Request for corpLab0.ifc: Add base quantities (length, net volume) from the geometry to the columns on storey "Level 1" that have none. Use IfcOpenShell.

First a look at what the model holds.

```python
import ifcopenshell
import ifcopenshell.util.element
import ifcopenshell.util.unit

model = ifcopenshell.open("corpLab0.ifc")
print(model.schema)
for unit_type in ("LENGTHUNIT", "AREAUNIT", "VOLUMEUNIT"):
    print(unit_type, ifcopenshell.util.unit.calculate_unit_scale(model, unit_type))
storey = next(s for s in model.by_type("IfcBuildingStorey") if s.Name == "Level 1")
columns = [e for e in ifcopenshell.util.element.get_decomposition(storey) if e.is_a("IfcColumn")]
for e in sorted(columns, key=lambda e: e.id()):
    print(e.id(), e.is_a(), e.Name, list(ifcopenshell.util.element.get_psets(e, qtos_only=True)), sep=" | ")
```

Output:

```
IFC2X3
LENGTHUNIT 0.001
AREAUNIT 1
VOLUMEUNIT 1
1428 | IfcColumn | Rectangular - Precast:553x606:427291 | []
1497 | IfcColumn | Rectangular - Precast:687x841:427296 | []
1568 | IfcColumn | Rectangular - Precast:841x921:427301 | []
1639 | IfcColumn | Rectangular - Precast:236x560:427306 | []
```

```python
import ifcopenshell
import ifcopenshell.api.pset
import ifcopenshell.geom
import ifcopenshell.util.element
import ifcopenshell.util.shape
import ifcopenshell.util.unit

model = ifcopenshell.open("corpLab0.ifc")
unit_scale = ifcopenshell.util.unit.calculate_unit_scale(model)
volume_scale = ifcopenshell.util.unit.calculate_unit_scale(model, "VOLUMEUNIT")
settings = ifcopenshell.geom.settings()

storey = next(s for s in model.by_type("IfcBuildingStorey") if s.Name == "Level 1")
columns = [e for e in ifcopenshell.util.element.get_decomposition(storey) if e.is_a("IfcColumn")]

for e in sorted(columns, key=lambda e: e.id()):
    if ifcopenshell.util.element.get_psets(e, qtos_only=True, should_inherit=False):
        continue
    # Geometry comes back in metres, in the element's own axes.
    shape = ifcopenshell.geom.create_shape(settings, e)
    values = {
        "Length": ifcopenshell.util.shape.get_z(shape.geometry) / unit_scale,
        "NetVolume": ifcopenshell.util.shape.get_volume(shape.geometry) / volume_scale,
    }
    qto = ifcopenshell.api.pset.add_qto(model, product=e, name="BaseQuantities")
    ifcopenshell.api.pset.edit_qto(model, qto=qto, properties=values)
    print(e.id(), {k: round(v, 3) for k, v in values.items()})

model.write("corpLab0_v2.ifc")
```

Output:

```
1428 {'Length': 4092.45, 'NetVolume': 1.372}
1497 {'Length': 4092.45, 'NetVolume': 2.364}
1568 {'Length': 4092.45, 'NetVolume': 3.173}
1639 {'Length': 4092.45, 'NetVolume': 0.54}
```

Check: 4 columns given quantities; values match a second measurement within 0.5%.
